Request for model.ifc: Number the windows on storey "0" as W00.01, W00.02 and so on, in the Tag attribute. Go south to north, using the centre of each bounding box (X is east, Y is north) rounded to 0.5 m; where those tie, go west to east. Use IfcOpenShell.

First a look at what the model holds.

```python
import ifcopenshell
import ifcopenshell.util.element
import ifcopenshell.util.placement

model = ifcopenshell.open("model.ifc")
print(model.schema)
storey = next(s for s in model.by_type("IfcBuildingStorey") if s.Name == "0")
windows = [e for e in ifcopenshell.util.element.get_decomposition(storey) if e.is_a("IfcWindow")]
for e in sorted(windows, key=lambda e: e.id()):
    origin = ifcopenshell.util.placement.get_local_placement(e.ObjectPlacement)[:3, 3]
    print(e.id(), e.Tag, e.Name, origin.round(2) + 0.0, sep=" | ")
```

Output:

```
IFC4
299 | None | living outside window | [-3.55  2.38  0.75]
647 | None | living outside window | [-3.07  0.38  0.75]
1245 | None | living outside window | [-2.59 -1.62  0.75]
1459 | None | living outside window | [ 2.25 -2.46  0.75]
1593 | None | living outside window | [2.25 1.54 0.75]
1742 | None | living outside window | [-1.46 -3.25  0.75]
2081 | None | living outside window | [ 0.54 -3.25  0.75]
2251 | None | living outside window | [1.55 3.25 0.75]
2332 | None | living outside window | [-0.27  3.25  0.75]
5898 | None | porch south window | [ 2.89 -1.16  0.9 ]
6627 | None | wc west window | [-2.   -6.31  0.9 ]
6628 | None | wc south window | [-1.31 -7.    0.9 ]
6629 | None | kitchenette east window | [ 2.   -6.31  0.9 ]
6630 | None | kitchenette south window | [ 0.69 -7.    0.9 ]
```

```python
import ifcopenshell
import ifcopenshell.geom
import ifcopenshell.util.element
import ifcopenshell.util.shape

model = ifcopenshell.open("model.ifc")
settings = ifcopenshell.geom.settings()
settings.set("use-world-coords", True)


def centre(element):
    shape = ifcopenshell.geom.create_shape(settings, element)
    return ifcopenshell.util.shape.get_bbox_centroid(shape.geometry)


storey = next(s for s in model.by_type("IfcBuildingStorey") if s.Name == "0")
windows = [e for e in ifcopenshell.util.element.get_decomposition(storey) if e.is_a("IfcWindow")]

# Insertion points can sit at a corner or the storey origin, so sort by the geometry (in metres).
centres = {e: centre(e) for e in windows}
windows.sort(key=lambda e: (round(centres[e][1] / 0.5), centres[e][0]))

for i, e in enumerate(windows, start=1):
    number = f"W00.{i:02d}"
    e.Tag = number
    print(e.id(), number)

model.write("model_rev.ifc")
```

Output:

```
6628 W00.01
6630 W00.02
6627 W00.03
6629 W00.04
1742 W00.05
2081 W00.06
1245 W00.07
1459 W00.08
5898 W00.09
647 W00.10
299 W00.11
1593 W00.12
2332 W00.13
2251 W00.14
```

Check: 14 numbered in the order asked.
